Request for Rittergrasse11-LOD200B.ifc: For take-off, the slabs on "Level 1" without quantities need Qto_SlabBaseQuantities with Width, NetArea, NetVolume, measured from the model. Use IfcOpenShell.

First a look at what the model holds.

```python
import ifcopenshell
import ifcopenshell.util.element
import ifcopenshell.util.unit

model = ifcopenshell.open("Rittergrasse11-LOD200B.ifc")
print(model.schema)
for unit_type in ("LENGTHUNIT", "AREAUNIT", "VOLUMEUNIT"):
    print(unit_type, ifcopenshell.util.unit.calculate_unit_scale(model, unit_type))
storey = next(s for s in model.by_type("IfcBuildingStorey") if s.Name == "Level 1")
slabs = [e for e in ifcopenshell.util.element.get_decomposition(storey) if e.is_a("IfcSlab")]
for e in sorted(slabs, key=lambda e: e.id()):
    print(e.id(), e.is_a(), e.Name, list(ifcopenshell.util.element.get_psets(e, qtos_only=True)), sep=" | ")
```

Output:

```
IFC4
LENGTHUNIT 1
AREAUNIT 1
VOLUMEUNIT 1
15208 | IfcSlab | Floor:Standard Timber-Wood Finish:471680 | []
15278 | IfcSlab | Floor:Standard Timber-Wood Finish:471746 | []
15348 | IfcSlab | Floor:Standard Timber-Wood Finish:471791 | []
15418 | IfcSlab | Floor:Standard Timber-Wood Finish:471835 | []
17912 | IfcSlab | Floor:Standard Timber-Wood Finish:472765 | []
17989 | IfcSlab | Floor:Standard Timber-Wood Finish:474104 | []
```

```python
import ifcopenshell
import ifcopenshell.api.pset
import ifcopenshell.geom
import ifcopenshell.util.element
import ifcopenshell.util.shape
import ifcopenshell.util.unit

model = ifcopenshell.open("Rittergrasse11-LOD200B.ifc")
unit_scale = ifcopenshell.util.unit.calculate_unit_scale(model)
area_scale = ifcopenshell.util.unit.calculate_unit_scale(model, "AREAUNIT")
volume_scale = ifcopenshell.util.unit.calculate_unit_scale(model, "VOLUMEUNIT")
settings = ifcopenshell.geom.settings()

storey = next(s for s in model.by_type("IfcBuildingStorey") if s.Name == "Level 1")
slabs = [e for e in ifcopenshell.util.element.get_decomposition(storey) if e.is_a("IfcSlab")]

for e in sorted(slabs, key=lambda e: e.id()):
    if ifcopenshell.util.element.get_psets(e, qtos_only=True, should_inherit=False):
        continue
    # Geometry comes back in metres, in the element's own axes.
    shape = ifcopenshell.geom.create_shape(settings, e)
    values = {
        "Width": ifcopenshell.util.shape.get_z(shape.geometry) / unit_scale,
        "NetArea": ifcopenshell.util.shape.get_footprint_area(shape.geometry) / area_scale,
        "NetVolume": ifcopenshell.util.shape.get_volume(shape.geometry) / volume_scale,
    }
    qto = ifcopenshell.api.pset.add_qto(model, product=e, name="Qto_SlabBaseQuantities")
    ifcopenshell.api.pset.edit_qto(model, qto=qto, properties=values)
    print(e.id(), {k: round(v, 3) for k, v in values.items()})

model.write("Rittergrasse11-LOD200B_edited.ifc")
```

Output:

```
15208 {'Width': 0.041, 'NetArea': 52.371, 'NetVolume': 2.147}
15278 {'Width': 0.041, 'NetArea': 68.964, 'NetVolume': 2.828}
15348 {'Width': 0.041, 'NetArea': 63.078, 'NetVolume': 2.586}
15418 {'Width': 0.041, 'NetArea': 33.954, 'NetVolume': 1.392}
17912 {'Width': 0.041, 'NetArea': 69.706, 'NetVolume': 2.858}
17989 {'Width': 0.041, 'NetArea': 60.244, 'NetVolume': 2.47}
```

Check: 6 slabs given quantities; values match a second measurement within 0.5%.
